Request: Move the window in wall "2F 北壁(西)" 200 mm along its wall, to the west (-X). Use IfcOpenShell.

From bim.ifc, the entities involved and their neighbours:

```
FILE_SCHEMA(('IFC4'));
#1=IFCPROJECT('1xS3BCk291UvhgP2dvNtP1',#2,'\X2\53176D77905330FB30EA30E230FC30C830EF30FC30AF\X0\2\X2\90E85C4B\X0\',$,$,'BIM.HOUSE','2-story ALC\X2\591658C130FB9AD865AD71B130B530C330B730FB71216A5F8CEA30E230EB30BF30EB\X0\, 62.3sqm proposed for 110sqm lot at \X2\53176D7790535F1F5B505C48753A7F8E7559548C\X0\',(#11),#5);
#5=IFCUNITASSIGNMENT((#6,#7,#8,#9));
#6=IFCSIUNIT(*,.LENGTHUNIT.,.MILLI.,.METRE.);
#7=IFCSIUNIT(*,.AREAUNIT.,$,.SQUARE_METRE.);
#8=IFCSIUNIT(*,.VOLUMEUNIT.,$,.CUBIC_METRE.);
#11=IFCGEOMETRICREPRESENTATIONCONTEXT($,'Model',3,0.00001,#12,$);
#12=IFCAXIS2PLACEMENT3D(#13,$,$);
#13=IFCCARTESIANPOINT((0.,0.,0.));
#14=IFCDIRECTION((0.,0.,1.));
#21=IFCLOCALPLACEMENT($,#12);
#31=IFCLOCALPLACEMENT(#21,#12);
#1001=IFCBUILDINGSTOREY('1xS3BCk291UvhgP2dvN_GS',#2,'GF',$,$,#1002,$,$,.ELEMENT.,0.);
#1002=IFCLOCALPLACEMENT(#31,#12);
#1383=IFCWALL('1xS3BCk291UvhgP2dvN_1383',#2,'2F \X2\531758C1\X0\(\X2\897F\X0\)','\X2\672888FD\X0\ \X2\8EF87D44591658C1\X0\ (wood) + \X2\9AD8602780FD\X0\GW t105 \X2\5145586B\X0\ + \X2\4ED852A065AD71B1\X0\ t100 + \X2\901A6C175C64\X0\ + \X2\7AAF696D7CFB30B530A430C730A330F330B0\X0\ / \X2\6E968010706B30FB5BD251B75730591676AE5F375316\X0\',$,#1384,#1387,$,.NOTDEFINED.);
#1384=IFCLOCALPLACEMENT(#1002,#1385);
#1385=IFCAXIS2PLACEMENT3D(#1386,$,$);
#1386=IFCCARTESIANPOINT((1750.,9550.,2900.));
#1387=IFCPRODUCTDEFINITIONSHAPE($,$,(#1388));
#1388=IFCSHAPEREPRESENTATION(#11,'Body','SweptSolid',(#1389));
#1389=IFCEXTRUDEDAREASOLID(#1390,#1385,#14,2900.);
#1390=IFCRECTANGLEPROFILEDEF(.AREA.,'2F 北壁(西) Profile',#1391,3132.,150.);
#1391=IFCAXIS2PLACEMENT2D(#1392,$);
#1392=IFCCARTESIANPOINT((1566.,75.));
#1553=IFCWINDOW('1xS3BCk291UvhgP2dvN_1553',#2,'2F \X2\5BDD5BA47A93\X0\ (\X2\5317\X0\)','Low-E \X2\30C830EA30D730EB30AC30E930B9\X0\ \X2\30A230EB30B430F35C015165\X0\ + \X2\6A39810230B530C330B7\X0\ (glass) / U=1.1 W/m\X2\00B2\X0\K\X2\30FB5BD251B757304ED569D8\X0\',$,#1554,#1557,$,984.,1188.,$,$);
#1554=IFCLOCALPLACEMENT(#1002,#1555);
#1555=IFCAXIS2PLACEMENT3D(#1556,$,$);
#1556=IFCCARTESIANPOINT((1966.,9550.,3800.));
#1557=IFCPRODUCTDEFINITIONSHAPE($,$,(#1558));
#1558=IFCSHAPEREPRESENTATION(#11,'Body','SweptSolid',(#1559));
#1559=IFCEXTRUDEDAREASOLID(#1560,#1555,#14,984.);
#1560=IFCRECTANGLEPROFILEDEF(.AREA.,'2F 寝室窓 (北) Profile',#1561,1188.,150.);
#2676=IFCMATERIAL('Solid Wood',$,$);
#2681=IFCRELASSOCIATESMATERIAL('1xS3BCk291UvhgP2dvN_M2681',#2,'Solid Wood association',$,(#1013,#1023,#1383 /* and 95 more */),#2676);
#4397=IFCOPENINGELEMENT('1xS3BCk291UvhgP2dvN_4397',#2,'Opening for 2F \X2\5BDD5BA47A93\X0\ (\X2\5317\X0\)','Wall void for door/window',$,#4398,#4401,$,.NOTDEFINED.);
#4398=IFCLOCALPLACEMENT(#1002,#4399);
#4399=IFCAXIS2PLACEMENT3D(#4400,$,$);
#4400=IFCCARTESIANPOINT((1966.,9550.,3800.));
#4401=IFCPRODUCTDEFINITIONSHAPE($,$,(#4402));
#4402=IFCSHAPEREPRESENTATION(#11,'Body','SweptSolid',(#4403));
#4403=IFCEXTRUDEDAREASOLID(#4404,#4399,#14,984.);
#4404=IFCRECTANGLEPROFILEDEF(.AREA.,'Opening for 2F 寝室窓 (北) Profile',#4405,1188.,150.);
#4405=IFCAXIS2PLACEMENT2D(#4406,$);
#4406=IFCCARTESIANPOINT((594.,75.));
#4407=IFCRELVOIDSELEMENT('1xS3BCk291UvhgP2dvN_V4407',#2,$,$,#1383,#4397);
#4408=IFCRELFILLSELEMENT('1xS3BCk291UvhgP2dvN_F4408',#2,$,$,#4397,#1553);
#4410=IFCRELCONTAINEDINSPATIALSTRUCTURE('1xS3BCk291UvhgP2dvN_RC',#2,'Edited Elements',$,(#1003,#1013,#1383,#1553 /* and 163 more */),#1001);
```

```python
import ifcopenshell
import ifcopenshell.api.geometry
import ifcopenshell.util.placement

model = ifcopenshell.open("bim.ifc")

window = model.by_guid("1xS3BCk291UvhgP2dvN_1553")
opening = window.FillsVoids[0].RelatingOpeningElement
wall = opening.VoidsElements[0].RelatingBuildingElement

wall_matrix = ifcopenshell.util.placement.get_local_placement(wall.ObjectPlacement)
shift = wall_matrix[:3, 0] * -200.0
before = ifcopenshell.util.placement.get_local_placement(window.ObjectPlacement)[:3, 3].copy()

# The window is not placed relative to its opening, so move both.
for product in (opening, window):
    matrix = ifcopenshell.util.placement.get_local_placement(product.ObjectPlacement)
    matrix[:3, 3] += shift
    ifcopenshell.api.geometry.edit_object_placement(model, product=product, matrix=matrix, is_si=False)

after = ifcopenshell.util.placement.get_local_placement(window.ObjectPlacement)[:3, 3]
print("window moved by", (after - before).round(3) + 0.0)

model.write("bim_updated.ifc")
```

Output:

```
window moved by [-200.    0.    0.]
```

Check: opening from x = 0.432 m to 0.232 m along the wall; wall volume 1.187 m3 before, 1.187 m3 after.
